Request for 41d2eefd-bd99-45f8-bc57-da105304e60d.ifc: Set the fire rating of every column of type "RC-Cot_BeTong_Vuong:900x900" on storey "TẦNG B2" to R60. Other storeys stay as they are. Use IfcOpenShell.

First a look at what the model holds.

```python
import ifcopenshell
import ifcopenshell.util.element

model = ifcopenshell.open("41d2eefd-bd99-45f8-bc57-da105304e60d.ifc")
print(model.schema)
storey = next(s for s in model.by_type("IfcBuildingStorey") if s.Name == "TẦNG B2")
columns = [e for e in ifcopenshell.util.element.get_decomposition(storey) if e.is_a("IfcColumn")]
seen = {}
for e in columns:
    element_type = ifcopenshell.util.element.get_type(e)
    key = (element_type.Name if element_type != e and element_type else None, ifcopenshell.util.element.get_pset(e, "Pset_ColumnCommon", "FireRating"))
    seen[key] = seen.get(key, 0) + 1
for (name, value), count in sorted(seen.items(), key=str):
    print(count, "x", name, "|", value)
```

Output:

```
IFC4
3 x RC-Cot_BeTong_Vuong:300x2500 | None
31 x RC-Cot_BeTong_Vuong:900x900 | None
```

```python
import ifcopenshell
import ifcopenshell.api.pset
import ifcopenshell.util.element

model = ifcopenshell.open("41d2eefd-bd99-45f8-bc57-da105304e60d.ifc")

storey = next(s for s in model.by_type("IfcBuildingStorey") if s.Name == "TẦNG B2")
columns = [e for e in ifcopenshell.util.element.get_decomposition(storey) if e.is_a("IfcColumn")]

count = 0
for e in columns:
    element_type = ifcopenshell.util.element.get_type(e)
    if element_type in (None, e) or element_type.Name != "RC-Cot_BeTong_Vuong:900x900":
        continue
    # add_pset returns the element's existing set when there is one.
    pset = ifcopenshell.api.pset.add_pset(model, product=e, name="Pset_ColumnCommon")
    ifcopenshell.api.pset.edit_pset(model, pset=pset, properties={"FireRating": "R60"})
    count += 1

print(count, "columns updated")

model.write("41d2eefd-bd99-45f8-bc57-da105304e60d_updated.ifc")
```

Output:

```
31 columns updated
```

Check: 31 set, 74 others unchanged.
